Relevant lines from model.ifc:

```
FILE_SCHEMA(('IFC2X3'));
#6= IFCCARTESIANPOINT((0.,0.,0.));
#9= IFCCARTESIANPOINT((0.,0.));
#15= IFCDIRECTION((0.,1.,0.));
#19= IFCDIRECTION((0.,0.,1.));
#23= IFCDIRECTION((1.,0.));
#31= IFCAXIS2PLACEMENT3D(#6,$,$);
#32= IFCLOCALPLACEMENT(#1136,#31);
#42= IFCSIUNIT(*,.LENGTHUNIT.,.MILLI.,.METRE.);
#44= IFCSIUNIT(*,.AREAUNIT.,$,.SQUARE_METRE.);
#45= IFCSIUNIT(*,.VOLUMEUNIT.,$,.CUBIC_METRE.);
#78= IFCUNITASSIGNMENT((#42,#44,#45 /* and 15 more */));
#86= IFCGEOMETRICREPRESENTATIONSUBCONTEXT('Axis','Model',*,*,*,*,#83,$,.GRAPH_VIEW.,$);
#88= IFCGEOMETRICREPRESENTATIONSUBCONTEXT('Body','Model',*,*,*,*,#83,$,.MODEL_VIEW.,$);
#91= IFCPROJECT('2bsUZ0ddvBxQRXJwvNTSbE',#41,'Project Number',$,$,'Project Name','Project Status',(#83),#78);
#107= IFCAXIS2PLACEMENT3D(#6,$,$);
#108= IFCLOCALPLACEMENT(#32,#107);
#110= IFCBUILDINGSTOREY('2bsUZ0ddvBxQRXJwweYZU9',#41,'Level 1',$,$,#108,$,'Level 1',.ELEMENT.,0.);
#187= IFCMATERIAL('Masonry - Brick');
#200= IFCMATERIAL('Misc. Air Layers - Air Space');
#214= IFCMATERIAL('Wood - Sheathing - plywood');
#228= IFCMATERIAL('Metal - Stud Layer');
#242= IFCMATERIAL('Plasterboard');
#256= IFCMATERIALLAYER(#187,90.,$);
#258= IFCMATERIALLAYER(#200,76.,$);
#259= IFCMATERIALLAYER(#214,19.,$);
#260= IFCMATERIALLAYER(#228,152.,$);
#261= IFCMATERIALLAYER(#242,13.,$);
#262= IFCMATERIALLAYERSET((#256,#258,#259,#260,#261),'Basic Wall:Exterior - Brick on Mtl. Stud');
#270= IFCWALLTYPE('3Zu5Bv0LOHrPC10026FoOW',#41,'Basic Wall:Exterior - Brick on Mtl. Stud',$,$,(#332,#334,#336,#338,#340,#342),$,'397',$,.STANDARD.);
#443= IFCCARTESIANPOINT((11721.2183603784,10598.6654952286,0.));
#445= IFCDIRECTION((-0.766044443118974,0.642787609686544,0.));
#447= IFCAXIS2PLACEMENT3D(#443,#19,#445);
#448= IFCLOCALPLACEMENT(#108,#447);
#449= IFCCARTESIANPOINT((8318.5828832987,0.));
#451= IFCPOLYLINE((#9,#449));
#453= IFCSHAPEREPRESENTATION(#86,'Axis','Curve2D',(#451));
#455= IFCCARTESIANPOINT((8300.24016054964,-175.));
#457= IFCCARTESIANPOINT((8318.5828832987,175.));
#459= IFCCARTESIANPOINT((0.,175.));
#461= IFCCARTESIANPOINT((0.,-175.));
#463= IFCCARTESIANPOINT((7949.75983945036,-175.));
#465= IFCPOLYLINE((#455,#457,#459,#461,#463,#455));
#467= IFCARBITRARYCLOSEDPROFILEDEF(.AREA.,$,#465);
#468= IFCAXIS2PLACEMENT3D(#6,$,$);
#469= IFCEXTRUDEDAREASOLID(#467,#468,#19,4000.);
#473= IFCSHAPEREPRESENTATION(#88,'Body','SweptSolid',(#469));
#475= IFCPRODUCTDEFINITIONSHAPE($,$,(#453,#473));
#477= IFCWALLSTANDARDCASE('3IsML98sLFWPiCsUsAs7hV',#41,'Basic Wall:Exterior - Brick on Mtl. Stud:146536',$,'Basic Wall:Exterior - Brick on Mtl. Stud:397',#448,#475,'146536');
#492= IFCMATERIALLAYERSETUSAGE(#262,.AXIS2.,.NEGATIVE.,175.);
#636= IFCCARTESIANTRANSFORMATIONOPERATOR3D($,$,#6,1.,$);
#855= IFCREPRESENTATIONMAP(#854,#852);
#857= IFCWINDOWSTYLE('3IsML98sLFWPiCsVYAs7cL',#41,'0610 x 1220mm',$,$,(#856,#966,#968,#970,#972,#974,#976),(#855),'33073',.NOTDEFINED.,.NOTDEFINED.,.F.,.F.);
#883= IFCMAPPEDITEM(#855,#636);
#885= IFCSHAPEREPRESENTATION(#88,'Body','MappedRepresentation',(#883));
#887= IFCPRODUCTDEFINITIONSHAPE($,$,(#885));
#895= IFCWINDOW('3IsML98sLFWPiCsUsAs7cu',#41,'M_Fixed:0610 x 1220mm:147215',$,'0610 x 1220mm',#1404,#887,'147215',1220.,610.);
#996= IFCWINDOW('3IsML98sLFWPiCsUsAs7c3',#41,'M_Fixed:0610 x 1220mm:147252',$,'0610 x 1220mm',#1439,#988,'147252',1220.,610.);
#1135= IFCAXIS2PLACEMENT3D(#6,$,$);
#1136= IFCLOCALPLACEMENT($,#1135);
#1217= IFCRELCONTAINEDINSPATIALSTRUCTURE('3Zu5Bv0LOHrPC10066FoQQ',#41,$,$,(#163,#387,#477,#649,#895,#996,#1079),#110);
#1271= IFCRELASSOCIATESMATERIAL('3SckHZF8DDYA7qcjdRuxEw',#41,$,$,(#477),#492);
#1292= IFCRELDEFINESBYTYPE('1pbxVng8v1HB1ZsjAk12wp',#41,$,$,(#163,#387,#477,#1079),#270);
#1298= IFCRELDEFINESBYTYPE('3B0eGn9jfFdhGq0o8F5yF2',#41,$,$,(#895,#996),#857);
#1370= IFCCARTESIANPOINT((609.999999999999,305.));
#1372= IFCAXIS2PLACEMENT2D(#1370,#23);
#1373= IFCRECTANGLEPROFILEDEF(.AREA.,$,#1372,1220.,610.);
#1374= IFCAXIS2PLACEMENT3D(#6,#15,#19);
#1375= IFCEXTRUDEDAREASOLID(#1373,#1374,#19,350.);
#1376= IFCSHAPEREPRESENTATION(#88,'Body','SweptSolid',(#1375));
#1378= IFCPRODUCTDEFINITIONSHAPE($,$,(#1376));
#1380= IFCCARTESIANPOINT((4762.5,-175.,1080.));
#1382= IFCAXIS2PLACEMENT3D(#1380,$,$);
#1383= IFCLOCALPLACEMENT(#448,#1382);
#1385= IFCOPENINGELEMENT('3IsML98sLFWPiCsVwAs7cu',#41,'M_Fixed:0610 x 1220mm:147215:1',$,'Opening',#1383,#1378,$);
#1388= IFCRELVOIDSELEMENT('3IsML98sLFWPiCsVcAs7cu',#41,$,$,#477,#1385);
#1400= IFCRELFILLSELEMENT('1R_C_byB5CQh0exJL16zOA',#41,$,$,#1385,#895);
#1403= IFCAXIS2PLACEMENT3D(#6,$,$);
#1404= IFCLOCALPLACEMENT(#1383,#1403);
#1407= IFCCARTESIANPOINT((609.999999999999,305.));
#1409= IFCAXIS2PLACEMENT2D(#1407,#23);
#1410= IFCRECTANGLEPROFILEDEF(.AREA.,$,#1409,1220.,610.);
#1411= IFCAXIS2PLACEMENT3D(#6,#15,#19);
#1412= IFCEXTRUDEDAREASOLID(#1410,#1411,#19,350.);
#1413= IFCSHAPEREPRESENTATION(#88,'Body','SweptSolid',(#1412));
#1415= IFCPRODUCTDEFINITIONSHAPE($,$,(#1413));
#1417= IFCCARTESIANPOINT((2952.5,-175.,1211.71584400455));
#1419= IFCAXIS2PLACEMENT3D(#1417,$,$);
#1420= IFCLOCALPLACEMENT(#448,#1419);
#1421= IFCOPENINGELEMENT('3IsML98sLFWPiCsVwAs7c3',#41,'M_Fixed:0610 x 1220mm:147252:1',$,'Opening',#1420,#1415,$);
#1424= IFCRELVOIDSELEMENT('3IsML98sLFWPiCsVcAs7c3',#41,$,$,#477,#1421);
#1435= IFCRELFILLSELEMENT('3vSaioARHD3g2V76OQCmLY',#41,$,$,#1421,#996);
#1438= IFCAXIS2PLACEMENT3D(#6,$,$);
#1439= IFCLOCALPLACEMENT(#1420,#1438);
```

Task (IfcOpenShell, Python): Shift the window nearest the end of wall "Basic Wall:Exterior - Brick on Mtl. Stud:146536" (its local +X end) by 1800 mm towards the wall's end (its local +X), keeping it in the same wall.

```python
import ifcopenshell
import ifcopenshell.api.geometry
import ifcopenshell.util.placement
import ifcopenshell.util.unit

model = ifcopenshell.open("model.ifc")
unit_scale = ifcopenshell.util.unit.calculate_unit_scale(model)

window = model.by_guid("3IsML98sLFWPiCsUsAs7cu")
opening = window.FillsVoids[0].RelatingOpeningElement
wall = opening.VoidsElements[0].RelatingBuildingElement

wall_matrix = ifcopenshell.util.placement.get_local_placement(wall.ObjectPlacement)
shift = wall_matrix[:3, 0] * 1.8 / unit_scale
before = ifcopenshell.util.placement.get_local_placement(window.ObjectPlacement)[:3, 3].copy()

# The window is placed relative to its opening, so it follows when the opening moves.
matrix = ifcopenshell.util.placement.get_local_placement(opening.ObjectPlacement)
matrix[:3, 3] += shift
ifcopenshell.api.geometry.edit_object_placement(
    model, product=opening, matrix=matrix, is_si=False, should_transform_children=True
)

after = ifcopenshell.util.placement.get_local_placement(window.ObjectPlacement)[:3, 3]
print("window moved by", (after - before).round(3) + 0.0)

model.write("model-out.ifc")
```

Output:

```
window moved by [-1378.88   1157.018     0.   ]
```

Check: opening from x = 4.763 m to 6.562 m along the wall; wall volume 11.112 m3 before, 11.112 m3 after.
